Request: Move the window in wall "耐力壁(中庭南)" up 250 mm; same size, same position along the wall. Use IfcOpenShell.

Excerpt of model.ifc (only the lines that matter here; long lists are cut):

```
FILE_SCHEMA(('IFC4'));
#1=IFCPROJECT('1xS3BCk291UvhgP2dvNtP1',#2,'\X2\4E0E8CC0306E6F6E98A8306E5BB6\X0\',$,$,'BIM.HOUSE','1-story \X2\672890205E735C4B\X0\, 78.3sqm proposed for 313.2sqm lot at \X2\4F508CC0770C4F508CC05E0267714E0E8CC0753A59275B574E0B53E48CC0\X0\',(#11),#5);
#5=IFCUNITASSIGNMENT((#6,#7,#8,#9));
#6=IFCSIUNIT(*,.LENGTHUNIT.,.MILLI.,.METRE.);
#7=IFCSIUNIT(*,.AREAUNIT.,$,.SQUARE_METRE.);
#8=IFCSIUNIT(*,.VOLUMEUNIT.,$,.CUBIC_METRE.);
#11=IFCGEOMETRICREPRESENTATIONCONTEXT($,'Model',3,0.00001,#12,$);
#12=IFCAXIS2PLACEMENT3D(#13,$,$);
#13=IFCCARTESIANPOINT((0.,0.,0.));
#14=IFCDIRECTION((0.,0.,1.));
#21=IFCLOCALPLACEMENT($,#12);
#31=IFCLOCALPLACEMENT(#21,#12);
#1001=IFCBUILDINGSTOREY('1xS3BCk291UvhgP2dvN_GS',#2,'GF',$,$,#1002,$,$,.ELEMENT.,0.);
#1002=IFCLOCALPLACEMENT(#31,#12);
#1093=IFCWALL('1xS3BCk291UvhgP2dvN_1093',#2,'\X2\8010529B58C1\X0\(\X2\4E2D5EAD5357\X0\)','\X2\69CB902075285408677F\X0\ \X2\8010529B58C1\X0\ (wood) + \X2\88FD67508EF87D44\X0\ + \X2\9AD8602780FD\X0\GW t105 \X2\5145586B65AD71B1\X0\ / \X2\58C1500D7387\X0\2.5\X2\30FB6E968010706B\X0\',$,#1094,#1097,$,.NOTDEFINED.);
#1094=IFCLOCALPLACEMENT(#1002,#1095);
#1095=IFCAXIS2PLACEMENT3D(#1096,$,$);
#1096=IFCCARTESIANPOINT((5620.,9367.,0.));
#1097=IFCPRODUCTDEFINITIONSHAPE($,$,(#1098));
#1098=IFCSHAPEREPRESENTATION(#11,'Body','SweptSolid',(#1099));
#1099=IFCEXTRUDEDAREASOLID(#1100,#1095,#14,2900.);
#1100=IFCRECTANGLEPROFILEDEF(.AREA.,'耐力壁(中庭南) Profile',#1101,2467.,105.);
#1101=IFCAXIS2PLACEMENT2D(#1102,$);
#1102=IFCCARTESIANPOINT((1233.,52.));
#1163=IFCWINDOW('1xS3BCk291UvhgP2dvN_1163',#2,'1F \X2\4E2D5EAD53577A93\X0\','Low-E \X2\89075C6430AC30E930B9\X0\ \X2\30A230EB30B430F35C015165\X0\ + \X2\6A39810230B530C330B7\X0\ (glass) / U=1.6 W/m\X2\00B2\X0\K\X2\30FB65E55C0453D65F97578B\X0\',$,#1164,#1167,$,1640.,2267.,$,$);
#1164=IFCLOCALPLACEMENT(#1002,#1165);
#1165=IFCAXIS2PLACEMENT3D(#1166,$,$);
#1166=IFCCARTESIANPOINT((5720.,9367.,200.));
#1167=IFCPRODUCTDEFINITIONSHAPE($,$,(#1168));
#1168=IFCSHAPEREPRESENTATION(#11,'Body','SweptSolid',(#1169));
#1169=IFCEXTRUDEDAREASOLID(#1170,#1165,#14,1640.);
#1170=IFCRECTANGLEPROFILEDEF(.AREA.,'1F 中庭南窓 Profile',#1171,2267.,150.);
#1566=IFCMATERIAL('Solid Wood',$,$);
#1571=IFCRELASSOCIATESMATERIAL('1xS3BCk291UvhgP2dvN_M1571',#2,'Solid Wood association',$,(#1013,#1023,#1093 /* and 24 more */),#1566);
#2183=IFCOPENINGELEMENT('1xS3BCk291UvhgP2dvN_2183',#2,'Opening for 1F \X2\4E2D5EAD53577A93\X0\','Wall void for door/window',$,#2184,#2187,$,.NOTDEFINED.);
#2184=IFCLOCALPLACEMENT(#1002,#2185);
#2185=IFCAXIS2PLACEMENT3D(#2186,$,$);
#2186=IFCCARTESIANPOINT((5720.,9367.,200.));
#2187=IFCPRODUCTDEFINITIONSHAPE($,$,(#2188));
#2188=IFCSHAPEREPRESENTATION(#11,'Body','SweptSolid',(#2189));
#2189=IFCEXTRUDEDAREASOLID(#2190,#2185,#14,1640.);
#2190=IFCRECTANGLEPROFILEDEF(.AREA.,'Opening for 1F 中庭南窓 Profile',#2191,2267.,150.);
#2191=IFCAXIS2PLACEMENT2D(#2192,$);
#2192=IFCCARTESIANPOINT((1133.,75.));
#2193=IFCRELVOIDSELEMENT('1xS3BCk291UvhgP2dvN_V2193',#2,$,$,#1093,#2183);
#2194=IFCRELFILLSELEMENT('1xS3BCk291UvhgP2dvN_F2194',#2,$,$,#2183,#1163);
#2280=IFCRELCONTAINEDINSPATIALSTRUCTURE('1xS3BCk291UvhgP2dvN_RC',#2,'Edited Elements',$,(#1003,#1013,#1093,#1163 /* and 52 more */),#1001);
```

```python
import numpy as np
import ifcopenshell
import ifcopenshell.api.geometry
import ifcopenshell.util.placement
import ifcopenshell.util.unit

model = ifcopenshell.open("model.ifc")
unit_scale = ifcopenshell.util.unit.calculate_unit_scale(model)

window = model.by_guid("1xS3BCk291UvhgP2dvN_1163")
opening = window.FillsVoids[0].RelatingOpeningElement
dz = 250.0

shift = np.array([0.0, 0.0, dz])
# The window is not placed relative to its opening, so move both.
for product in (opening, window):
    matrix = ifcopenshell.util.placement.get_local_placement(product.ObjectPlacement)
    matrix[:3, 3] += shift
    ifcopenshell.api.geometry.edit_object_placement(model, product=product, matrix=matrix, is_si=False)

print(f"moved by {dz * unit_scale:+.3f} m")

model.write("model_updated.ifc")
```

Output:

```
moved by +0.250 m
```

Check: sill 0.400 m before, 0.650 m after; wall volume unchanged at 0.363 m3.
